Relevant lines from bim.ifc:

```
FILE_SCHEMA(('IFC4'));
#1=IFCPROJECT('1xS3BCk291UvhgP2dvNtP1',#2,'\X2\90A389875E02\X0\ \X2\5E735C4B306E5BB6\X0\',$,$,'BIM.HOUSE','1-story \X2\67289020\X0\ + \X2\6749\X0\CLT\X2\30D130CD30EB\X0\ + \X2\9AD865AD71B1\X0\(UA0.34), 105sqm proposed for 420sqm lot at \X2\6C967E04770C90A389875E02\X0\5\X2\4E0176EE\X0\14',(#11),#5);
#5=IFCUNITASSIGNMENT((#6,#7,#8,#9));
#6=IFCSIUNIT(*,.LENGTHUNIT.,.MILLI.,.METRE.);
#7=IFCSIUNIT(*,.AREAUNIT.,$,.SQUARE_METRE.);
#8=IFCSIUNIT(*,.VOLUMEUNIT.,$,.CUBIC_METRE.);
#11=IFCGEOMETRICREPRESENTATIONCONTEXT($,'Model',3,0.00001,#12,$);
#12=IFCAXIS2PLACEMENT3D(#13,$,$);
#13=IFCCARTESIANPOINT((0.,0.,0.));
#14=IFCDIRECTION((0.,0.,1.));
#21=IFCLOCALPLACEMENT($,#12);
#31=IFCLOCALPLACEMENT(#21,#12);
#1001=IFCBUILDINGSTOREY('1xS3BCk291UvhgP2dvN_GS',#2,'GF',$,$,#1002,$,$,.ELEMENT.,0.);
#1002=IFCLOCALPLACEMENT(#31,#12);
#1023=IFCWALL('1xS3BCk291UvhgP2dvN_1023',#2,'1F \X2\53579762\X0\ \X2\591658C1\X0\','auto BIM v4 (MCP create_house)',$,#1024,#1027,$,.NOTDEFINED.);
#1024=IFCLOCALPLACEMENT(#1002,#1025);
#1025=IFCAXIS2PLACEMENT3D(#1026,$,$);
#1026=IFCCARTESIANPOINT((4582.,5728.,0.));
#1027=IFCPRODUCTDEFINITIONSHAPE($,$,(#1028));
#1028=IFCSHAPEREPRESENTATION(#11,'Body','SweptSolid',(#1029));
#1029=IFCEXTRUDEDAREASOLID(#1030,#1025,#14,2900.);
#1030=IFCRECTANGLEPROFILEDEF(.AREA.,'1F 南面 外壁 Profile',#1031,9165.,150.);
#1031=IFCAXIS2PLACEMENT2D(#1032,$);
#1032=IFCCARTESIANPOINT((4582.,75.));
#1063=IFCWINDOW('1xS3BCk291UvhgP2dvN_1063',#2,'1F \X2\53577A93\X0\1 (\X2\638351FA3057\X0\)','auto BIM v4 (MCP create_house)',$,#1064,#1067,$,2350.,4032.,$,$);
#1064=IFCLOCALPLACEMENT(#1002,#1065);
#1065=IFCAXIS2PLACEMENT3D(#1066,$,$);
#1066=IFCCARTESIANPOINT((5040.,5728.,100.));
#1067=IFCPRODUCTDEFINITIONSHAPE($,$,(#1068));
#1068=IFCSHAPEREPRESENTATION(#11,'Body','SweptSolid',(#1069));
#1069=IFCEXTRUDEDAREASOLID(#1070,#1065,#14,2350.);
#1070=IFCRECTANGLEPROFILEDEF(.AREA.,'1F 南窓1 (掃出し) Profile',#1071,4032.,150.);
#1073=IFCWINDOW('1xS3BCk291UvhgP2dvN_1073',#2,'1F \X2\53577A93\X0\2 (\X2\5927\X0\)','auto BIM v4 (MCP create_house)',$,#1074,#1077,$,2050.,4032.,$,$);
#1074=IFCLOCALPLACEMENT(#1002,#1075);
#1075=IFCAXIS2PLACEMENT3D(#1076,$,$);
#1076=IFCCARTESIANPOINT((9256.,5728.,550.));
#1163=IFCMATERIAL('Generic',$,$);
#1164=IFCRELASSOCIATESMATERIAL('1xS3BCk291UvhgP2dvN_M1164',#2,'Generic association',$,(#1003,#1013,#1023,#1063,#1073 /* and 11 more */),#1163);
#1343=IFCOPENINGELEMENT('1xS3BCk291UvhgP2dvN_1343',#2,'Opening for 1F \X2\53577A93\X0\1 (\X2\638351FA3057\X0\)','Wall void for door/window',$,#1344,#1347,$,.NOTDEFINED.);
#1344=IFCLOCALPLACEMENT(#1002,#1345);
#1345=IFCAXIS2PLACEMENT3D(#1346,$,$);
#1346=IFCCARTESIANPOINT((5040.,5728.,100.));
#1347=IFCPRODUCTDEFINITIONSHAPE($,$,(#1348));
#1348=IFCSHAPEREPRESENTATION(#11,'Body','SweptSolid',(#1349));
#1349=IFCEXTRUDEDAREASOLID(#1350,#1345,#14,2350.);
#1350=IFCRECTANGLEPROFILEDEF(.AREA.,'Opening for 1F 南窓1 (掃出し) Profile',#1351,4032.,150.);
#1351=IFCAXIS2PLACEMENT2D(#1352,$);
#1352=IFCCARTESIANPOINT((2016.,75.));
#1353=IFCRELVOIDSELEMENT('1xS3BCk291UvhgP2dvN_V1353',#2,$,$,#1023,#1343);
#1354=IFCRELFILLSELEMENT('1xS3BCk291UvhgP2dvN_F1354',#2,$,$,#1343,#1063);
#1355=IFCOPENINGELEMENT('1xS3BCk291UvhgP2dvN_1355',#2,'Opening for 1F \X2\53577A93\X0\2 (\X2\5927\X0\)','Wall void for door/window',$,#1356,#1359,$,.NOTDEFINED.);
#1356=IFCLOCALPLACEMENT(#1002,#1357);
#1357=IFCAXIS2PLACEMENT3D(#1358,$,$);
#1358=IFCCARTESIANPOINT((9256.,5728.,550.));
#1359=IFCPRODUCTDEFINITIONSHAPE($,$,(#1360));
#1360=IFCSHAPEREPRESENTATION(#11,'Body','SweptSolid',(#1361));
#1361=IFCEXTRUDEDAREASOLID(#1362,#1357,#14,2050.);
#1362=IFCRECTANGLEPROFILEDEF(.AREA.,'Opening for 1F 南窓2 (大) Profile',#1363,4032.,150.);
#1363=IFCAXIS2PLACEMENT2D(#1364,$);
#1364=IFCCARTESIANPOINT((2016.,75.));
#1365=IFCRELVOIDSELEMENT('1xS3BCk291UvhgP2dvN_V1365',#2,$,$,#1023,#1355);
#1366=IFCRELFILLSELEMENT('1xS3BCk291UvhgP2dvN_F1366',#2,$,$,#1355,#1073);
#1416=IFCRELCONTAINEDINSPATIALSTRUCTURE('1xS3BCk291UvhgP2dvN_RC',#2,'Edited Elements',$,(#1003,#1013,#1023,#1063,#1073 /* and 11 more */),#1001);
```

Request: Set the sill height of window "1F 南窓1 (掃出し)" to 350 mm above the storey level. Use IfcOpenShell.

```python
import numpy as np
import ifcopenshell
import ifcopenshell.api.geometry
import ifcopenshell.geom
import ifcopenshell.util.element
import ifcopenshell.util.placement
import ifcopenshell.util.shape
import ifcopenshell.util.unit

model = ifcopenshell.open("bim.ifc")
unit_scale = ifcopenshell.util.unit.calculate_unit_scale(model)

window = model.by_guid("1xS3BCk291UvhgP2dvN_1063")
opening = window.FillsVoids[0].RelatingOpeningElement
storey = ifcopenshell.util.element.get_container(window, ifc_class="IfcBuildingStorey")
level = ifcopenshell.util.placement.get_local_placement(storey.ObjectPlacement)[2, 3]

# The opening's origin need not be at the sill, so measure its lowest point.
shape = ifcopenshell.geom.create_shape(ifcopenshell.geom.settings(), opening)
bottom = ifcopenshell.util.shape.get_shape_bottom_elevation(shape, shape.geometry) / unit_scale
dz = level + 0.35 / unit_scale - bottom

shift = np.array([0.0, 0.0, dz])
# The window is not placed relative to its opening, so move both.
for product in (opening, window):
    matrix = ifcopenshell.util.placement.get_local_placement(product.ObjectPlacement)
    matrix[:3, 3] += shift
    ifcopenshell.api.geometry.edit_object_placement(model, product=product, matrix=matrix, is_si=False)

print(f"moved by {dz * unit_scale:+.3f} m")

model.write("bim_rev.ifc")
```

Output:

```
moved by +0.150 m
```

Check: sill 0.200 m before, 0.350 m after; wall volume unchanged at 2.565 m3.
